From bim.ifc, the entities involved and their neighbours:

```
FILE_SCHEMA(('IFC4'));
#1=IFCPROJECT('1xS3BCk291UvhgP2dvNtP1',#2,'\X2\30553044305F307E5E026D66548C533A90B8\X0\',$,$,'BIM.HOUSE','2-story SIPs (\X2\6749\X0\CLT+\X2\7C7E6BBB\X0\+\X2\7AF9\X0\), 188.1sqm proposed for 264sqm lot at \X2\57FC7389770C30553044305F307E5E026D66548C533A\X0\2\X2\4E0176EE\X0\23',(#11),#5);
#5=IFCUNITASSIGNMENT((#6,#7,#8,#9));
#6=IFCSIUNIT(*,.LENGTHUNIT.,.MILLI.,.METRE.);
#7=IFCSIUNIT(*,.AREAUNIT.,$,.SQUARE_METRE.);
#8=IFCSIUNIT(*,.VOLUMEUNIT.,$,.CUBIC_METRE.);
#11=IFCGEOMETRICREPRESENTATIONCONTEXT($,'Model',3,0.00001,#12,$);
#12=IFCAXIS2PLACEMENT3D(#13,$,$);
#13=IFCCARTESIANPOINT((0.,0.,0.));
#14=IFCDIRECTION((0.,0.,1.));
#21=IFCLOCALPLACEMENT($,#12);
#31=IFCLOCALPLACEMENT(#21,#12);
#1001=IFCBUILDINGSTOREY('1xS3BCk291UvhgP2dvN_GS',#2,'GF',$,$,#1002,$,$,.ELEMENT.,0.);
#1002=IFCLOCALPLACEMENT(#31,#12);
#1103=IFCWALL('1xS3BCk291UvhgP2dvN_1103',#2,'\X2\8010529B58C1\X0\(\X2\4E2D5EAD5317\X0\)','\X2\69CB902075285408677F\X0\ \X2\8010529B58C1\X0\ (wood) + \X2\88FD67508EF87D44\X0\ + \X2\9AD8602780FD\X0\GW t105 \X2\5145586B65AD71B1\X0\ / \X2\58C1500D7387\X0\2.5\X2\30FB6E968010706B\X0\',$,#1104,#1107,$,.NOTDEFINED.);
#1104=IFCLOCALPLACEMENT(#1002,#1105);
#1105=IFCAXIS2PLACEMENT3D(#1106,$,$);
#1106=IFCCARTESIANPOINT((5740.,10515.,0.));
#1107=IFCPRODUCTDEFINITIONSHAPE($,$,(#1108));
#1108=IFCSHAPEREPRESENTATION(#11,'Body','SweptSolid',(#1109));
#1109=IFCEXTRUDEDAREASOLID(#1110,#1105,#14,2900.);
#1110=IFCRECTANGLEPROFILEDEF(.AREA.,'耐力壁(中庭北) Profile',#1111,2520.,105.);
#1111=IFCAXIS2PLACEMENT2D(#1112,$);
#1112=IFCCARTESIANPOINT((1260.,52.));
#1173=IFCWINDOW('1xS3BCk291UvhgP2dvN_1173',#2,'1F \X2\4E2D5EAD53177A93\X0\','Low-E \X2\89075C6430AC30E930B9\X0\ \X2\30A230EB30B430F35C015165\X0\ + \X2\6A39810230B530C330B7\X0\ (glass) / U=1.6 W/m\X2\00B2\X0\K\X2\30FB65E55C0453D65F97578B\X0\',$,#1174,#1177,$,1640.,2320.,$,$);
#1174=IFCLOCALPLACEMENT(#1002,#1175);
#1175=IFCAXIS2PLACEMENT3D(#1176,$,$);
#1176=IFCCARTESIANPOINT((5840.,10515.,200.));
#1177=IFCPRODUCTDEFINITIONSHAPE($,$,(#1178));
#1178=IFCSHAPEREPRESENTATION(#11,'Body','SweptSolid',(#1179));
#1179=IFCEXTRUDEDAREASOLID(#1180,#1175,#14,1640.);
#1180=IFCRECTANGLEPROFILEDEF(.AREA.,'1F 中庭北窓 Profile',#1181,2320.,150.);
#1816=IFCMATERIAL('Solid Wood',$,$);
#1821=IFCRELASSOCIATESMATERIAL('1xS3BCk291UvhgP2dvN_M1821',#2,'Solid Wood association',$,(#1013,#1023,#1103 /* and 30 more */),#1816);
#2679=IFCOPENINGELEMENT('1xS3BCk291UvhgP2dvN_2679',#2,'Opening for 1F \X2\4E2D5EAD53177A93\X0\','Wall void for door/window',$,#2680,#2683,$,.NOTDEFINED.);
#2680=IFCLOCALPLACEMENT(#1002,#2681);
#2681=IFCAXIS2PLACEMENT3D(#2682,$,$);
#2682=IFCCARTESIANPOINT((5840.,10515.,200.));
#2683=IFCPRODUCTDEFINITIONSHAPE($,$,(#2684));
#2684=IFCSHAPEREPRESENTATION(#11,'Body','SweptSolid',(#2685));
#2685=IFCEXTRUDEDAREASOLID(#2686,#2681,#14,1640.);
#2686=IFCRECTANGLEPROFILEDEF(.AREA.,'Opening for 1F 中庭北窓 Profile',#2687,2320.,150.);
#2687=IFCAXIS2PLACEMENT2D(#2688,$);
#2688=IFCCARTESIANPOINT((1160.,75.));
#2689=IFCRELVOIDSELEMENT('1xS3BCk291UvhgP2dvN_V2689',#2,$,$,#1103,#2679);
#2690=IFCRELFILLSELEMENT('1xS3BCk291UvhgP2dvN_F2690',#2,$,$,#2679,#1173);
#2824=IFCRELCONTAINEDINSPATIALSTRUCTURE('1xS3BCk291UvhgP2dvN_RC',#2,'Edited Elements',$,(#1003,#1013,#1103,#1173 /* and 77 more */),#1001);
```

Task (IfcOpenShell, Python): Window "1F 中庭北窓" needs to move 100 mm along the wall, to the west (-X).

```python
import ifcopenshell
import ifcopenshell.api.geometry
import ifcopenshell.util.placement
import ifcopenshell.util.unit

model = ifcopenshell.open("bim.ifc")
unit_scale = ifcopenshell.util.unit.calculate_unit_scale(model)

window = model.by_id(1173)
opening = window.FillsVoids[0].RelatingOpeningElement
wall = opening.VoidsElements[0].RelatingBuildingElement

wall_matrix = ifcopenshell.util.placement.get_local_placement(wall.ObjectPlacement)
shift = wall_matrix[:3, 0] * -0.1 / unit_scale
before = ifcopenshell.util.placement.get_local_placement(window.ObjectPlacement)[:3, 3].copy()

# The window is not placed relative to its opening, so move both.
for product in (opening, window):
    matrix = ifcopenshell.util.placement.get_local_placement(product.ObjectPlacement)
    matrix[:3, 3] += shift
    ifcopenshell.api.geometry.edit_object_placement(model, product=product, matrix=matrix, is_si=False)

after = ifcopenshell.util.placement.get_local_placement(window.ObjectPlacement)[:3, 3]
print("window moved by", (after - before).round(3) + 0.0)

model.write("bim_rev.ifc")
```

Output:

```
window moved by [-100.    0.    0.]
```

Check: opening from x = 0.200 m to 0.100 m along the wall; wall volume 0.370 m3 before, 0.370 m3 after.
